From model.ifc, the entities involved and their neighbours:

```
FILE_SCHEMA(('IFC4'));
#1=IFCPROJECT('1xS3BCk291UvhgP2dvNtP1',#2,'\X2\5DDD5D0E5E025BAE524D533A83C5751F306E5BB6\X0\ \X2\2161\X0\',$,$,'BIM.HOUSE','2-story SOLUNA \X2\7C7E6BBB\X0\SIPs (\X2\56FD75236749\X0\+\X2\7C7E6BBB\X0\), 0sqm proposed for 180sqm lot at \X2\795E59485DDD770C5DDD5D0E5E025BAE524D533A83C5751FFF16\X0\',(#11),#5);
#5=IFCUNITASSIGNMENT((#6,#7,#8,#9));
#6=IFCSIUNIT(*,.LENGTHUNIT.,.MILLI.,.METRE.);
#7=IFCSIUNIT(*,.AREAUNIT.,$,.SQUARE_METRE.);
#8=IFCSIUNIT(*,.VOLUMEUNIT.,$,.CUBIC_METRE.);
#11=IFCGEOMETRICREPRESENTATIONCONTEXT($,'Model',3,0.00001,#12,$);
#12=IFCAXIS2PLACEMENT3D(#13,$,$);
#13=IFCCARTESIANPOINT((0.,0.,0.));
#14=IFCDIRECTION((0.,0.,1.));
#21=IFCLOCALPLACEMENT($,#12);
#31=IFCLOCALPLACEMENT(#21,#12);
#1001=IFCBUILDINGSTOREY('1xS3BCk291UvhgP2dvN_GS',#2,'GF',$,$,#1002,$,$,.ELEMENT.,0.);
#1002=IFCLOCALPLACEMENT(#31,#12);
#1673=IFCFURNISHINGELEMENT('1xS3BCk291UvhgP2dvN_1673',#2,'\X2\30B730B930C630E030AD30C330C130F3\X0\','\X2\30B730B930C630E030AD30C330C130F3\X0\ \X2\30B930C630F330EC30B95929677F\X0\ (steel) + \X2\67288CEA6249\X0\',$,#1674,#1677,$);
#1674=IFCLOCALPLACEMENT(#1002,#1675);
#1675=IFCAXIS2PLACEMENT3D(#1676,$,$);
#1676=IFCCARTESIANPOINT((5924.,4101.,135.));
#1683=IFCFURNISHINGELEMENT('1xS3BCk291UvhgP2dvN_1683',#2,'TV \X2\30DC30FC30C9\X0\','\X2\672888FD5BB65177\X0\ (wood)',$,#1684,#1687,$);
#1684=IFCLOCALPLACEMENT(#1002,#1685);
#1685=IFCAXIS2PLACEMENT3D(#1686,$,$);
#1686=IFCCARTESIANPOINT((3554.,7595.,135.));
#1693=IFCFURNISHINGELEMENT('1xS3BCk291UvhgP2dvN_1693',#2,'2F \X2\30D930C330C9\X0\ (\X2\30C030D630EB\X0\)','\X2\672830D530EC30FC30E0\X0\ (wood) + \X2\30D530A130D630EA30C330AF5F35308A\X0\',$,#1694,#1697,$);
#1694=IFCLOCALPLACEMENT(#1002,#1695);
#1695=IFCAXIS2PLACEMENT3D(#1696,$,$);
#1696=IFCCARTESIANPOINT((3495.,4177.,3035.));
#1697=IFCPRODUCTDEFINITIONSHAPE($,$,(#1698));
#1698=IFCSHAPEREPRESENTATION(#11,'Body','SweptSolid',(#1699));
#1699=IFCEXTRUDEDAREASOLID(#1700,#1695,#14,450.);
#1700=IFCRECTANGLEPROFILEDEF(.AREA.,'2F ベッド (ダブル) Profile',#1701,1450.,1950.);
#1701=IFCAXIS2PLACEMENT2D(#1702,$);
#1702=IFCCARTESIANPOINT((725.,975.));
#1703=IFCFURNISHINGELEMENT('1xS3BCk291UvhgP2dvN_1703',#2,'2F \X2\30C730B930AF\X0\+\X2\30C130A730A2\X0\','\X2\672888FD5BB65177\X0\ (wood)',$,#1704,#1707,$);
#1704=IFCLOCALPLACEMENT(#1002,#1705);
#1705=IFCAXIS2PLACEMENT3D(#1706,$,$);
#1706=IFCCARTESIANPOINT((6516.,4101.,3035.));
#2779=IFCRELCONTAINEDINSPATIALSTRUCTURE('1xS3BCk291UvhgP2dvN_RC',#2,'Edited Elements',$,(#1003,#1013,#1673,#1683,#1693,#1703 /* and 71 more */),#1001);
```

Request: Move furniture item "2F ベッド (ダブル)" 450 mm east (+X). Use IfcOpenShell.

```python
import ifcopenshell
import ifcopenshell.api.geometry
import ifcopenshell.util.placement
import ifcopenshell.util.unit

model = ifcopenshell.open("model.ifc")
unit_scale = ifcopenshell.util.unit.calculate_unit_scale(model)

item = model.by_id(1693)
matrix = ifcopenshell.util.placement.get_local_placement(item.ObjectPlacement)
matrix[0, 3] += 0.45 / unit_scale
ifcopenshell.api.geometry.edit_object_placement(model, product=item, matrix=matrix, is_si=False)

print(ifcopenshell.util.placement.get_local_placement(item.ObjectPlacement).round(3) + 0.0)

model.write("model_updated.ifc")
```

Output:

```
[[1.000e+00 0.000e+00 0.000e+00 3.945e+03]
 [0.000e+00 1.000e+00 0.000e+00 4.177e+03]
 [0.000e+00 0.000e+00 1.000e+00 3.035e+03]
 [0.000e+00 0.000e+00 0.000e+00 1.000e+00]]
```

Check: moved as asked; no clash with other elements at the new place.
